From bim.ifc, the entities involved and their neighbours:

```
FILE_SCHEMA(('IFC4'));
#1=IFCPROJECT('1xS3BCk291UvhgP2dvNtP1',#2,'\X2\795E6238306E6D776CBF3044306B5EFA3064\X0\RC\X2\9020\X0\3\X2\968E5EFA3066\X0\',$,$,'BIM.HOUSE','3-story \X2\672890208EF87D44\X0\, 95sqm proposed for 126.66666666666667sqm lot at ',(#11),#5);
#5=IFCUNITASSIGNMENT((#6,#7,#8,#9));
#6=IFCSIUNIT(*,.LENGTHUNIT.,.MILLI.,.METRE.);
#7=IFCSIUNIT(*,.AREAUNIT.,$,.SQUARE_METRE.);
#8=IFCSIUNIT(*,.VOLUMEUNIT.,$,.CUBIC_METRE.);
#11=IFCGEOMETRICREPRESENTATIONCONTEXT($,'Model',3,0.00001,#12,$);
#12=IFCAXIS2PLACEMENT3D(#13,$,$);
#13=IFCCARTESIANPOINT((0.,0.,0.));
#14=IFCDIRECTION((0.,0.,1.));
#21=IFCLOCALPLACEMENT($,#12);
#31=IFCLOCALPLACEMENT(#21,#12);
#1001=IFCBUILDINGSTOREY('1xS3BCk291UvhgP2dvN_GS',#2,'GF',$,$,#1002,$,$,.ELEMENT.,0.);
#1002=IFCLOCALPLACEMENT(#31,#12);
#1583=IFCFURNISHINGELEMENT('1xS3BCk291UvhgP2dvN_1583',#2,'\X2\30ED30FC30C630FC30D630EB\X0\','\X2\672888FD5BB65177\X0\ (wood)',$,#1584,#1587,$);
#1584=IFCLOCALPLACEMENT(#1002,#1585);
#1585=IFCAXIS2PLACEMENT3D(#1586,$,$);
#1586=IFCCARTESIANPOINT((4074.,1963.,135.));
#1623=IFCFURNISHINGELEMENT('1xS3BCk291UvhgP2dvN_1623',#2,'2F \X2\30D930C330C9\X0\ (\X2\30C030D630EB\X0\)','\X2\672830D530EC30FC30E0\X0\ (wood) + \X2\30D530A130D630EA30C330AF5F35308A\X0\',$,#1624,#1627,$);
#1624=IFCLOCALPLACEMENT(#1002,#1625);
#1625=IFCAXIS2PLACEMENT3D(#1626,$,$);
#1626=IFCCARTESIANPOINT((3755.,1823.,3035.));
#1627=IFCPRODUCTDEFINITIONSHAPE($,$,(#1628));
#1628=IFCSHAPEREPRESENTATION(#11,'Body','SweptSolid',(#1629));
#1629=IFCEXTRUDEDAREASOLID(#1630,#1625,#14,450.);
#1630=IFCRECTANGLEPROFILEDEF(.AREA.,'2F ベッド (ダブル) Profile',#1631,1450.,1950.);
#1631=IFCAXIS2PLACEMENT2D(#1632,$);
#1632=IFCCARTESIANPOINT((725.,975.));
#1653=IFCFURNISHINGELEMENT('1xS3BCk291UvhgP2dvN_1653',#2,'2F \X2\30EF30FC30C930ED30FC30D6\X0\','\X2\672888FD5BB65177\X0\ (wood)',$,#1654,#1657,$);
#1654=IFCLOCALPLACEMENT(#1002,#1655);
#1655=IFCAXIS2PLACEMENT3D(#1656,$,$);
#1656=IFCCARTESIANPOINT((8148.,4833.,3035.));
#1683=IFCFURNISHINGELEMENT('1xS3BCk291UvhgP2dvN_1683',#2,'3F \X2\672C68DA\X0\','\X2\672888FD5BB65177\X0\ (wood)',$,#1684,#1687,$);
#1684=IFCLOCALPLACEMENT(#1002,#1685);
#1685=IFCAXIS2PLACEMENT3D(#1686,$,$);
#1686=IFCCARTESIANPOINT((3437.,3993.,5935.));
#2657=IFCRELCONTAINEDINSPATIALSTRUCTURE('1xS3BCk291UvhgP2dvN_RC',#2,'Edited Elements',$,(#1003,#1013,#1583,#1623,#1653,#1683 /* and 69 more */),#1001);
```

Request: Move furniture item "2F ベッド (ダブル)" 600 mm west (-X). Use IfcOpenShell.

```python
import ifcopenshell
import ifcopenshell.api.geometry
import ifcopenshell.util.placement
import ifcopenshell.util.unit

model = ifcopenshell.open("bim.ifc")
unit_scale = ifcopenshell.util.unit.calculate_unit_scale(model)

item = model.by_id(1623)
matrix = ifcopenshell.util.placement.get_local_placement(item.ObjectPlacement)
matrix[0, 3] -= 0.6 / unit_scale
ifcopenshell.api.geometry.edit_object_placement(model, product=item, matrix=matrix, is_si=False)

print(ifcopenshell.util.placement.get_local_placement(item.ObjectPlacement).round(3) + 0.0)

model.write("bim_updated.ifc")
```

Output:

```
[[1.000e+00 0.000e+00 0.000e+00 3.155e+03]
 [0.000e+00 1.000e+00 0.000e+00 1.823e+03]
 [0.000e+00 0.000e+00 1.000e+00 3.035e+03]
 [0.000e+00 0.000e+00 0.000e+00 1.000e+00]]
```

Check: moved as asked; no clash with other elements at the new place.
